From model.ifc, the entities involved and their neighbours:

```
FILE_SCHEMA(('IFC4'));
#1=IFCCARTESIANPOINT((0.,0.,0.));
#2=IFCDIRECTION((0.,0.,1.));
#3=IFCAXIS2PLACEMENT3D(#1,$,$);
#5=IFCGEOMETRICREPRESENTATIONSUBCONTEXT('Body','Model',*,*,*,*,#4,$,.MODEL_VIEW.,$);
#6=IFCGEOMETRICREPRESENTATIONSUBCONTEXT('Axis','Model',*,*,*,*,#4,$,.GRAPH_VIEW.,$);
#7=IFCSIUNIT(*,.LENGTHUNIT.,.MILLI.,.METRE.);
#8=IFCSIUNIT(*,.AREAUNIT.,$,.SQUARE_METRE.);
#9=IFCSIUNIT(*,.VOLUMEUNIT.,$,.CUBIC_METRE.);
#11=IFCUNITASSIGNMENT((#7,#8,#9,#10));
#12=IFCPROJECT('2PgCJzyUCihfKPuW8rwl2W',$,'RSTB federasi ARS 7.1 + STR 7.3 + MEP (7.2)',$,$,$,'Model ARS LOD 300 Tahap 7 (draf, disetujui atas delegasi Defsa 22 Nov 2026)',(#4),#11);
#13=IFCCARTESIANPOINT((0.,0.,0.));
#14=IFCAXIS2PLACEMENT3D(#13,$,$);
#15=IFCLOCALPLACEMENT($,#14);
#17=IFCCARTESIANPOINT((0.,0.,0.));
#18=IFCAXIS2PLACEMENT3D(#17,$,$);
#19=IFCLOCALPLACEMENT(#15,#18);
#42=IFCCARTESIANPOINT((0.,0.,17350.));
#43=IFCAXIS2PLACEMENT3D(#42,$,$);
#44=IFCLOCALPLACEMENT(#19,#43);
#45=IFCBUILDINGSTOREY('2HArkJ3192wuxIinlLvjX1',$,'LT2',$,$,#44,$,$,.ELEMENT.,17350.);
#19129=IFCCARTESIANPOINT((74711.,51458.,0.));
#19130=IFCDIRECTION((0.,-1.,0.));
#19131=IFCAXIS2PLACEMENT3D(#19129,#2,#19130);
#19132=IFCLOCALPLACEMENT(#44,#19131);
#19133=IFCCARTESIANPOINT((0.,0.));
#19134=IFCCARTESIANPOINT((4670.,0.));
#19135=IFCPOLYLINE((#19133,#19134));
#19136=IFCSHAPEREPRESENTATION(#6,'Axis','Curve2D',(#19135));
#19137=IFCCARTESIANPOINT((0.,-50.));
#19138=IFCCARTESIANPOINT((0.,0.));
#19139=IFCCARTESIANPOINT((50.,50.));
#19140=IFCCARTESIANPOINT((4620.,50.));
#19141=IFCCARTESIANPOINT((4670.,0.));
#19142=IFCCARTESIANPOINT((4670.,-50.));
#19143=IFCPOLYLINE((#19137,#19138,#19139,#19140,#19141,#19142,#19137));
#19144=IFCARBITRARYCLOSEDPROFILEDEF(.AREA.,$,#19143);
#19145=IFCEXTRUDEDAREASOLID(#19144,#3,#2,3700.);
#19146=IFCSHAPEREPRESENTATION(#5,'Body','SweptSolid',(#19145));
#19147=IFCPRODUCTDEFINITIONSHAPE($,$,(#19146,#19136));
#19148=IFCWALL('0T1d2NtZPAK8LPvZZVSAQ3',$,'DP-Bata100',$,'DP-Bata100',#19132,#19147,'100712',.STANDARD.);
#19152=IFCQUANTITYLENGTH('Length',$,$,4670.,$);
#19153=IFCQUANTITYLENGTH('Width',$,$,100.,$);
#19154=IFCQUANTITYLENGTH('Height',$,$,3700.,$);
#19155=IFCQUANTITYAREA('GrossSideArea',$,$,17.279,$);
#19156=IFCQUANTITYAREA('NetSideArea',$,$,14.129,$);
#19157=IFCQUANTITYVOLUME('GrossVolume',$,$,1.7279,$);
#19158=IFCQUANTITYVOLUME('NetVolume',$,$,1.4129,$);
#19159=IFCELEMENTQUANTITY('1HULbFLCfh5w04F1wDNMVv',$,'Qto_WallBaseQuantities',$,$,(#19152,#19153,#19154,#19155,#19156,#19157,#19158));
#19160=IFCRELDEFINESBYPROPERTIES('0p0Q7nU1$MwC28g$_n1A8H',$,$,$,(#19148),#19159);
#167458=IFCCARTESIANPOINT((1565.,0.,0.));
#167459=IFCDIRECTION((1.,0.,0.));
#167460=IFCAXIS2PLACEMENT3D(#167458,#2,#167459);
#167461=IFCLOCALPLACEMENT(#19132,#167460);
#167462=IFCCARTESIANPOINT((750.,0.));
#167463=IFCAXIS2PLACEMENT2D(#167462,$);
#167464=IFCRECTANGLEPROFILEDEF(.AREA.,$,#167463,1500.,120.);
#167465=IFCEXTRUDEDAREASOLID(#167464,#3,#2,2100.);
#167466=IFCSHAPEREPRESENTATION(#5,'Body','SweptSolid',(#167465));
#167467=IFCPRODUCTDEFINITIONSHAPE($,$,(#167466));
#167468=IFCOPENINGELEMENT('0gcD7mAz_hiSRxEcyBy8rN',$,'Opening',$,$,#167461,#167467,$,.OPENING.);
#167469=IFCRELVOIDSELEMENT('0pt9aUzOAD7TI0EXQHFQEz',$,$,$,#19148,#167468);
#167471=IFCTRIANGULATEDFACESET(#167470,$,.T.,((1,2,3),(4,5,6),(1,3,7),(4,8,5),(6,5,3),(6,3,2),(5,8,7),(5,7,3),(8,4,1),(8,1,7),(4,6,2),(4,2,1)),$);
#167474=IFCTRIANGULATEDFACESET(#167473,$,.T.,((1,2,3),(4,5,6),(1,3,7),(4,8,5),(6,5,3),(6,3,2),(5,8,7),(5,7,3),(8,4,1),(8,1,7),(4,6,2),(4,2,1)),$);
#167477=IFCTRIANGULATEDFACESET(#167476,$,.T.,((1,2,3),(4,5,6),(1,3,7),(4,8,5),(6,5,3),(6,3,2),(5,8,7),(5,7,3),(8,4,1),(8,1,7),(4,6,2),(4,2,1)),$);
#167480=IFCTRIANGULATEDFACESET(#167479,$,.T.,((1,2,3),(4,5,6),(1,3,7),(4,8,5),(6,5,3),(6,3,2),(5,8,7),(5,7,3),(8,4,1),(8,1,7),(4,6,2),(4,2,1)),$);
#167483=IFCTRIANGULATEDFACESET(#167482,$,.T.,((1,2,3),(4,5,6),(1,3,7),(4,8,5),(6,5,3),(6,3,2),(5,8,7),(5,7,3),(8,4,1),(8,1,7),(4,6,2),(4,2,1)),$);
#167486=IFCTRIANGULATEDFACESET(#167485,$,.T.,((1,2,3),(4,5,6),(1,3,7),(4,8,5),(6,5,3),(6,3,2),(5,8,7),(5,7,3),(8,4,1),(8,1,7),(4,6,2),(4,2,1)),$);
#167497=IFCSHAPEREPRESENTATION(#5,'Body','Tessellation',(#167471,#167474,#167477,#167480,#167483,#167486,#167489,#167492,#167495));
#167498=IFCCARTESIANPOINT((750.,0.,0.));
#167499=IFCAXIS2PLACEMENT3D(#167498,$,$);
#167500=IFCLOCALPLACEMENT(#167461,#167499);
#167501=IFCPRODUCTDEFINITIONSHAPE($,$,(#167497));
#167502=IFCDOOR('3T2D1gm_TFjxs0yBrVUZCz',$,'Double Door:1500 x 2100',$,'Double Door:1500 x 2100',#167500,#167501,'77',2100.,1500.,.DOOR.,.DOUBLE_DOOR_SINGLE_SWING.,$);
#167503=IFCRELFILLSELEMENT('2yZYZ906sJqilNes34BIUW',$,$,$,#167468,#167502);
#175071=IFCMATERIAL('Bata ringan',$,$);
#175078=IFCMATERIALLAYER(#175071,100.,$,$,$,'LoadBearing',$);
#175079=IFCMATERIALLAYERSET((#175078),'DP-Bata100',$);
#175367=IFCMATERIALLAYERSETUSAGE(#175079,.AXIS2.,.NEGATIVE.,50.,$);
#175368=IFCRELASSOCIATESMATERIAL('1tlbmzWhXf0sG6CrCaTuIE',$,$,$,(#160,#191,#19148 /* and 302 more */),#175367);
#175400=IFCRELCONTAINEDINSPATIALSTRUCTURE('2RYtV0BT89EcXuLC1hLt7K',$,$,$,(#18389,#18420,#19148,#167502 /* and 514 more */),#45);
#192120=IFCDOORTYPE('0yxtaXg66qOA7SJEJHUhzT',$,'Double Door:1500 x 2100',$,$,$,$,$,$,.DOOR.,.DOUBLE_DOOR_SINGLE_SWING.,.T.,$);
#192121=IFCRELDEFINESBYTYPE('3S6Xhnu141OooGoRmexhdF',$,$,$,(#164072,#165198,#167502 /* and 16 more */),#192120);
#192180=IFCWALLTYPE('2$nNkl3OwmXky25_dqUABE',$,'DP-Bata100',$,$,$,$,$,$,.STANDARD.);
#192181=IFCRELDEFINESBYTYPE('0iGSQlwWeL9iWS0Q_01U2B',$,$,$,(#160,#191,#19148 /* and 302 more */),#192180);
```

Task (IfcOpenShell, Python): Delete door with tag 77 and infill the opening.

```python
import ifcopenshell
import ifcopenshell.api.feature
import ifcopenshell.api.pset
import ifcopenshell.api.root
import ifcopenshell.geom
import ifcopenshell.util.element
import ifcopenshell.util.shape
import ifcopenshell.util.unit

model = ifcopenshell.open("model.ifc")
area_scale = ifcopenshell.util.unit.calculate_unit_scale(model, "AREAUNIT")
volume_scale = ifcopenshell.util.unit.calculate_unit_scale(model, "VOLUMEUNIT")
settings = ifcopenshell.geom.settings()


def volume(element):
    """Net volume in cubic metres, openings subtracted."""
    shape = ifcopenshell.geom.create_shape(settings, element)
    return ifcopenshell.util.shape.get_volume(shape.geometry)


door = model.by_guid("3T2D1gm_TFjxs0yBrVUZCz")
opening = door.FillsVoids[0].RelatingOpeningElement
wall = opening.VoidsElements[0].RelatingBuildingElement
before = volume(wall)

ifcopenshell.api.root.remove_product(model, product=door)
ifcopenshell.api.feature.remove_feature(model, feature=opening)

after = volume(wall)
thickness = 0.1  # wall thickness in metres

# Update the wall's stored quantities.
qto = model.by_id(ifcopenshell.util.element.get_pset(wall, "Qto_WallBaseQuantities", should_inherit=False)["id"])
ifcopenshell.api.pset.edit_qto(model, qto=qto, properties={
    "NetSideArea": after / thickness / area_scale,
    "NetVolume": after / volume_scale,
})

print(f"wall volume {before:.3f} -> {after:.3f} m3")

model.write("model_v2.ifc")
```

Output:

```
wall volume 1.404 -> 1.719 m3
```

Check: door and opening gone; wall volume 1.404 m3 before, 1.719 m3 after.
